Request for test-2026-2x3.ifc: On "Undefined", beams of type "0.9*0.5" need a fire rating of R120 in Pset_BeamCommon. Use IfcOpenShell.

First a look at what the model holds.

```python
import ifcopenshell
import ifcopenshell.util.element

model = ifcopenshell.open("test-2026-2x3.ifc")
print(model.schema)
storey = next(s for s in model.by_type("IfcBuildingStorey") if s.Name == "Undefined")
beams = [e for e in ifcopenshell.util.element.get_decomposition(storey) if e.is_a("IfcBeam")]
seen = {}
for e in beams:
    element_type = ifcopenshell.util.element.get_type(e)
    key = (element_type.Name if element_type != e and element_type else None, ifcopenshell.util.element.get_pset(e, "Pset_BeamCommon", "FireRating"))
    seen[key] = seen.get(key, 0) + 1
for (name, value), count in sorted(seen.items(), key=str):
    print(count, "x", name, "|", value)
```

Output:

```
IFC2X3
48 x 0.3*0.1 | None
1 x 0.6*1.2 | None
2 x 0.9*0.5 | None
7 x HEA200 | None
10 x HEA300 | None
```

```python
import ifcopenshell
import ifcopenshell.api.pset
import ifcopenshell.util.element

model = ifcopenshell.open("test-2026-2x3.ifc")

storey = next(s for s in model.by_type("IfcBuildingStorey") if s.Name == "Undefined")
beams = [e for e in ifcopenshell.util.element.get_decomposition(storey) if e.is_a("IfcBeam")]

count = 0
for e in beams:
    element_type = ifcopenshell.util.element.get_type(e)
    if element_type in (None, e) or element_type.Name != "0.9*0.5":
        continue
    # add_pset returns the element's existing set when there is one.
    pset = ifcopenshell.api.pset.add_pset(model, product=e, name="Pset_BeamCommon")
    ifcopenshell.api.pset.edit_pset(model, pset=pset, properties={"FireRating": "R120"})
    count += 1

print(count, "beams updated")

model.write("test-2026-2x3-out.ifc")
```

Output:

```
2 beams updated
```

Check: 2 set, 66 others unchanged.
